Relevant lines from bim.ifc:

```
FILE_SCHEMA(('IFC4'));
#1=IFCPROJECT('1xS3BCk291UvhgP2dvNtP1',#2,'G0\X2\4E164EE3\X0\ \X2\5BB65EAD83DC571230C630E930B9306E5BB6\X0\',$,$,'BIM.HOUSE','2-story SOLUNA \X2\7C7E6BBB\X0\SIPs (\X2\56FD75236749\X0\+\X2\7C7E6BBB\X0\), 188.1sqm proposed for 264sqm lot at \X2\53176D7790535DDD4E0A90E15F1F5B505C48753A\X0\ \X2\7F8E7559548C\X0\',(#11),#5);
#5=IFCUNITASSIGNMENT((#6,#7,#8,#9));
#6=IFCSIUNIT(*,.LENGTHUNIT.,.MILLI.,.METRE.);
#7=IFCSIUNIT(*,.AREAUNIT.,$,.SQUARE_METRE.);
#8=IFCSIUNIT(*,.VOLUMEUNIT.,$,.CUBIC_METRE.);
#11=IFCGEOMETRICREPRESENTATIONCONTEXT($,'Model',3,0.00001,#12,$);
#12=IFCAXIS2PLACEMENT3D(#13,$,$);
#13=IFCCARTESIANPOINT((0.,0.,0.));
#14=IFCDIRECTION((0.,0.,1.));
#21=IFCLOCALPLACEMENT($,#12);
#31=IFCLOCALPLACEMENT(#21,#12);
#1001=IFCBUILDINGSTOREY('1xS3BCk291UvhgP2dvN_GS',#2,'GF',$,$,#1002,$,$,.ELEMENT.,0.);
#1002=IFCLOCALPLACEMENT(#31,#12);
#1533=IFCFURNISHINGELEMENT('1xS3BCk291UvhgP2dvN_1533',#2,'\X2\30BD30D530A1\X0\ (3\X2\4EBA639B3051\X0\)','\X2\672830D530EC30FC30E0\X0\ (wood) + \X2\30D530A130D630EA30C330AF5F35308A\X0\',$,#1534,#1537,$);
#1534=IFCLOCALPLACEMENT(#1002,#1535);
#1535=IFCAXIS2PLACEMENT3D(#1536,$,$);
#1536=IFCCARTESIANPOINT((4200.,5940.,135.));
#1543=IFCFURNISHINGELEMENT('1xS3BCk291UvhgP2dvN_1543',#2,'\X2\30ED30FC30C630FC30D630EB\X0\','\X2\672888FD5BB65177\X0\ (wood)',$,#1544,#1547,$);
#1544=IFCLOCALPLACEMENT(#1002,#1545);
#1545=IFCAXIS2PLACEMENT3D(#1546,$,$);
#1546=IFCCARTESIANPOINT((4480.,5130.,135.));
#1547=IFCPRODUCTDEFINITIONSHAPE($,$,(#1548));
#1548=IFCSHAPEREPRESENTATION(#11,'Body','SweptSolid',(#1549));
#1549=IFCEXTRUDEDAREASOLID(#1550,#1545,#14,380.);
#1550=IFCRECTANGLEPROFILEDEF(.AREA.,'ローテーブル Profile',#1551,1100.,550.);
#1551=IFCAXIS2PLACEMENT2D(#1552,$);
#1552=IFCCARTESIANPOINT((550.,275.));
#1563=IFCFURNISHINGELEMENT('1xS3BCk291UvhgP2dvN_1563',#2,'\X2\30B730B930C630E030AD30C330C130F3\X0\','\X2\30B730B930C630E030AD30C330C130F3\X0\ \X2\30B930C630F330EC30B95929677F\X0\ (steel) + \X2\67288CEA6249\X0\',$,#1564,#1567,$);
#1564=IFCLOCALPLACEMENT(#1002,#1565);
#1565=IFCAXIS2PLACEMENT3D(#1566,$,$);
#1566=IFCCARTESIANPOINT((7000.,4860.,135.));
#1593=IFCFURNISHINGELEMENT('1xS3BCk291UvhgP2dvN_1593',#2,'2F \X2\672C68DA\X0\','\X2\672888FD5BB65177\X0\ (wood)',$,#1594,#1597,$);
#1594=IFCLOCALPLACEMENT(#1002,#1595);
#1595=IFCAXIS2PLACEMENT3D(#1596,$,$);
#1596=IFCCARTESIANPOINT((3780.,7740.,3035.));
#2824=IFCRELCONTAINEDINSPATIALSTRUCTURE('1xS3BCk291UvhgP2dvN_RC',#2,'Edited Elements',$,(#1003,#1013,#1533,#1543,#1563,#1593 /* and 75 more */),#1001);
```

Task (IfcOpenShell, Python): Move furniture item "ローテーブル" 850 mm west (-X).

```python
import ifcopenshell
import ifcopenshell.api.geometry
import ifcopenshell.util.placement
import ifcopenshell.util.unit

model = ifcopenshell.open("bim.ifc")
unit_scale = ifcopenshell.util.unit.calculate_unit_scale(model)

item = model.by_guid("1xS3BCk291UvhgP2dvN_1543")
matrix = ifcopenshell.util.placement.get_local_placement(item.ObjectPlacement)
matrix[0, 3] -= 0.85 / unit_scale
ifcopenshell.api.geometry.edit_object_placement(model, product=item, matrix=matrix, is_si=False)

print(ifcopenshell.util.placement.get_local_placement(item.ObjectPlacement).round(3) + 0.0)

model.write("bim_rev.ifc")
```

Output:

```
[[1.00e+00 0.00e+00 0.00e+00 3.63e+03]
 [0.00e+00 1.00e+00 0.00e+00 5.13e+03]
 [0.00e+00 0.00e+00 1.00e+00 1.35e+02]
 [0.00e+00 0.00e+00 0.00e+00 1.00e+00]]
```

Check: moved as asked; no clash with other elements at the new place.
